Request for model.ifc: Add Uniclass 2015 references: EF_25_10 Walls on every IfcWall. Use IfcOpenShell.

First a look at what the model holds.

```python
import ifcopenshell

model = ifcopenshell.open("model.ifc")
print(model.schema)
print("classifications:", [c.Name for c in model.by_type("IfcClassification")])
for ifc_class in ("IfcDoor", "IfcRoof", "IfcStair", "IfcWall", "IfcWindow"):
    print(ifc_class, len(model.by_type(ifc_class)))
```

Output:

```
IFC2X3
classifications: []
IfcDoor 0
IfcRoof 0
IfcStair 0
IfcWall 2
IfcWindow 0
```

```python
import ifcopenshell
import ifcopenshell.api.classification

model = ifcopenshell.open("model.ifc")

# IFC2X3 requires Source and Edition and has no link from the project to the system.
system = model.create_entity("IfcClassification", Source="NBS", Edition="2015", Name="Uniclass 2015")

codes = {
    "IfcWall": ("EF_25_10", "Walls"),
}
for ifc_class, (code, name) in codes.items():
    products = model.by_type(ifc_class)
    ifcopenshell.api.classification.add_reference(
        model, products=products, classification=system, identification=code, name=name
    )
    print(code, len(products))

model.write("model_v2.ifc")
```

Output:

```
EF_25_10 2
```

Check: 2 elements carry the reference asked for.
